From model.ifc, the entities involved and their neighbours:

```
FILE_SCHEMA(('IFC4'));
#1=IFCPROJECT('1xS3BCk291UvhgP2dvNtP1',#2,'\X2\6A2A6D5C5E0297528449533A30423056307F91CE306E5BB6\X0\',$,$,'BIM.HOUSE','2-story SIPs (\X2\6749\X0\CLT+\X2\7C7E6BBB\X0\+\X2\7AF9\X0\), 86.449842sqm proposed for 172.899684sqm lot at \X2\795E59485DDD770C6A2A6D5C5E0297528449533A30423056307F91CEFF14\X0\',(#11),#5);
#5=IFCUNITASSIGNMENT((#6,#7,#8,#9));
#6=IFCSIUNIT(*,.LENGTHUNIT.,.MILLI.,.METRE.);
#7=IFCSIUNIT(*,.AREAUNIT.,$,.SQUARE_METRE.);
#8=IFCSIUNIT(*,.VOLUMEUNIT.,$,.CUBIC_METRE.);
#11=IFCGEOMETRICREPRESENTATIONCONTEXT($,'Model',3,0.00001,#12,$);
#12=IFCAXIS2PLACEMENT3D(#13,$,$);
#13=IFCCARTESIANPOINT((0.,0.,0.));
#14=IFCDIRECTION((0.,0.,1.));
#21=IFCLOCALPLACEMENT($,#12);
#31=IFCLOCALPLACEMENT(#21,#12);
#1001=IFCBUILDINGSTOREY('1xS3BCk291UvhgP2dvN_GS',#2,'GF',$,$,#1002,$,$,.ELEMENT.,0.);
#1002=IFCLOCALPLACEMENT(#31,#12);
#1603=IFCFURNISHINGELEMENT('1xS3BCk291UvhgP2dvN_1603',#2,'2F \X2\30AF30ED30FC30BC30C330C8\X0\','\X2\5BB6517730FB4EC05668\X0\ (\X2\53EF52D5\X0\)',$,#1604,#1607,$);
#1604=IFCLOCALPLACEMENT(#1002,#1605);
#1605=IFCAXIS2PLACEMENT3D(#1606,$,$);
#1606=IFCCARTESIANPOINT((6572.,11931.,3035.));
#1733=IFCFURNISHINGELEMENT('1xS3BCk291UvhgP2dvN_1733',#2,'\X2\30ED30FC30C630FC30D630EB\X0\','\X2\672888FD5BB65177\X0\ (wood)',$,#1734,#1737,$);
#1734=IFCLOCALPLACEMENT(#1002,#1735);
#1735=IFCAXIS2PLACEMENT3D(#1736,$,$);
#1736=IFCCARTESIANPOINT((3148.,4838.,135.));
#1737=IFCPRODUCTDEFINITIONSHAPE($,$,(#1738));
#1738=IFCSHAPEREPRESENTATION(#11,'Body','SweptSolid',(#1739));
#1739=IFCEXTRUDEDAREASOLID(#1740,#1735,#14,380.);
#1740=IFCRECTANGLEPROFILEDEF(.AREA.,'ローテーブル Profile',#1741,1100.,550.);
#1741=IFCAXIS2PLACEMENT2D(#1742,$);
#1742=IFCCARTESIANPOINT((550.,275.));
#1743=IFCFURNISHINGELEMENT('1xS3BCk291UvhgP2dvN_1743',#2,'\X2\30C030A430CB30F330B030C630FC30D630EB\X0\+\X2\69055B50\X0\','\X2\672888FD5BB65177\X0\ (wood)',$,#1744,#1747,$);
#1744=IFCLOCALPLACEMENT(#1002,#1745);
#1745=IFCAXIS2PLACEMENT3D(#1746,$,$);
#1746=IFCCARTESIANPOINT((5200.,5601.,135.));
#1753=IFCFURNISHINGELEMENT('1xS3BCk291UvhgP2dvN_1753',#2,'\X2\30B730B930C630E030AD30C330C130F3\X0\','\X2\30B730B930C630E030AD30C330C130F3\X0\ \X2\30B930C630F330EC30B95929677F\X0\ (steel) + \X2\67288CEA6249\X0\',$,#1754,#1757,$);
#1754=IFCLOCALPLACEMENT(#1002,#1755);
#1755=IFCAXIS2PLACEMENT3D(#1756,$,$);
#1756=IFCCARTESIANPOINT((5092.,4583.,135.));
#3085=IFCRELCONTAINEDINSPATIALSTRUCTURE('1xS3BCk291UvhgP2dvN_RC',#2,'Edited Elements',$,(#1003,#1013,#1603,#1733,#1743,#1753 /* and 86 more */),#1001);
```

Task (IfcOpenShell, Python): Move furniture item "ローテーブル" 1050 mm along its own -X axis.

```python
import ifcopenshell
import ifcopenshell.api.geometry
import ifcopenshell.util.placement

model = ifcopenshell.open("model.ifc")

item = model.by_id(1733)
matrix = ifcopenshell.util.placement.get_local_placement(item.ObjectPlacement)
matrix[:3, 3] -= matrix[:3, 0] * 1050.0
ifcopenshell.api.geometry.edit_object_placement(model, product=item, matrix=matrix, is_si=False)

print(ifcopenshell.util.placement.get_local_placement(item.ObjectPlacement).round(3) + 0.0)

model.write("model_rev.ifc")
```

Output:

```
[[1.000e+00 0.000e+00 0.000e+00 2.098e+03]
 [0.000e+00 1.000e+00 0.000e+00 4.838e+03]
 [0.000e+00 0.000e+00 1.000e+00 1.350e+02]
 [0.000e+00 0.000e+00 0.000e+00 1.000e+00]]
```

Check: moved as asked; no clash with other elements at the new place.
